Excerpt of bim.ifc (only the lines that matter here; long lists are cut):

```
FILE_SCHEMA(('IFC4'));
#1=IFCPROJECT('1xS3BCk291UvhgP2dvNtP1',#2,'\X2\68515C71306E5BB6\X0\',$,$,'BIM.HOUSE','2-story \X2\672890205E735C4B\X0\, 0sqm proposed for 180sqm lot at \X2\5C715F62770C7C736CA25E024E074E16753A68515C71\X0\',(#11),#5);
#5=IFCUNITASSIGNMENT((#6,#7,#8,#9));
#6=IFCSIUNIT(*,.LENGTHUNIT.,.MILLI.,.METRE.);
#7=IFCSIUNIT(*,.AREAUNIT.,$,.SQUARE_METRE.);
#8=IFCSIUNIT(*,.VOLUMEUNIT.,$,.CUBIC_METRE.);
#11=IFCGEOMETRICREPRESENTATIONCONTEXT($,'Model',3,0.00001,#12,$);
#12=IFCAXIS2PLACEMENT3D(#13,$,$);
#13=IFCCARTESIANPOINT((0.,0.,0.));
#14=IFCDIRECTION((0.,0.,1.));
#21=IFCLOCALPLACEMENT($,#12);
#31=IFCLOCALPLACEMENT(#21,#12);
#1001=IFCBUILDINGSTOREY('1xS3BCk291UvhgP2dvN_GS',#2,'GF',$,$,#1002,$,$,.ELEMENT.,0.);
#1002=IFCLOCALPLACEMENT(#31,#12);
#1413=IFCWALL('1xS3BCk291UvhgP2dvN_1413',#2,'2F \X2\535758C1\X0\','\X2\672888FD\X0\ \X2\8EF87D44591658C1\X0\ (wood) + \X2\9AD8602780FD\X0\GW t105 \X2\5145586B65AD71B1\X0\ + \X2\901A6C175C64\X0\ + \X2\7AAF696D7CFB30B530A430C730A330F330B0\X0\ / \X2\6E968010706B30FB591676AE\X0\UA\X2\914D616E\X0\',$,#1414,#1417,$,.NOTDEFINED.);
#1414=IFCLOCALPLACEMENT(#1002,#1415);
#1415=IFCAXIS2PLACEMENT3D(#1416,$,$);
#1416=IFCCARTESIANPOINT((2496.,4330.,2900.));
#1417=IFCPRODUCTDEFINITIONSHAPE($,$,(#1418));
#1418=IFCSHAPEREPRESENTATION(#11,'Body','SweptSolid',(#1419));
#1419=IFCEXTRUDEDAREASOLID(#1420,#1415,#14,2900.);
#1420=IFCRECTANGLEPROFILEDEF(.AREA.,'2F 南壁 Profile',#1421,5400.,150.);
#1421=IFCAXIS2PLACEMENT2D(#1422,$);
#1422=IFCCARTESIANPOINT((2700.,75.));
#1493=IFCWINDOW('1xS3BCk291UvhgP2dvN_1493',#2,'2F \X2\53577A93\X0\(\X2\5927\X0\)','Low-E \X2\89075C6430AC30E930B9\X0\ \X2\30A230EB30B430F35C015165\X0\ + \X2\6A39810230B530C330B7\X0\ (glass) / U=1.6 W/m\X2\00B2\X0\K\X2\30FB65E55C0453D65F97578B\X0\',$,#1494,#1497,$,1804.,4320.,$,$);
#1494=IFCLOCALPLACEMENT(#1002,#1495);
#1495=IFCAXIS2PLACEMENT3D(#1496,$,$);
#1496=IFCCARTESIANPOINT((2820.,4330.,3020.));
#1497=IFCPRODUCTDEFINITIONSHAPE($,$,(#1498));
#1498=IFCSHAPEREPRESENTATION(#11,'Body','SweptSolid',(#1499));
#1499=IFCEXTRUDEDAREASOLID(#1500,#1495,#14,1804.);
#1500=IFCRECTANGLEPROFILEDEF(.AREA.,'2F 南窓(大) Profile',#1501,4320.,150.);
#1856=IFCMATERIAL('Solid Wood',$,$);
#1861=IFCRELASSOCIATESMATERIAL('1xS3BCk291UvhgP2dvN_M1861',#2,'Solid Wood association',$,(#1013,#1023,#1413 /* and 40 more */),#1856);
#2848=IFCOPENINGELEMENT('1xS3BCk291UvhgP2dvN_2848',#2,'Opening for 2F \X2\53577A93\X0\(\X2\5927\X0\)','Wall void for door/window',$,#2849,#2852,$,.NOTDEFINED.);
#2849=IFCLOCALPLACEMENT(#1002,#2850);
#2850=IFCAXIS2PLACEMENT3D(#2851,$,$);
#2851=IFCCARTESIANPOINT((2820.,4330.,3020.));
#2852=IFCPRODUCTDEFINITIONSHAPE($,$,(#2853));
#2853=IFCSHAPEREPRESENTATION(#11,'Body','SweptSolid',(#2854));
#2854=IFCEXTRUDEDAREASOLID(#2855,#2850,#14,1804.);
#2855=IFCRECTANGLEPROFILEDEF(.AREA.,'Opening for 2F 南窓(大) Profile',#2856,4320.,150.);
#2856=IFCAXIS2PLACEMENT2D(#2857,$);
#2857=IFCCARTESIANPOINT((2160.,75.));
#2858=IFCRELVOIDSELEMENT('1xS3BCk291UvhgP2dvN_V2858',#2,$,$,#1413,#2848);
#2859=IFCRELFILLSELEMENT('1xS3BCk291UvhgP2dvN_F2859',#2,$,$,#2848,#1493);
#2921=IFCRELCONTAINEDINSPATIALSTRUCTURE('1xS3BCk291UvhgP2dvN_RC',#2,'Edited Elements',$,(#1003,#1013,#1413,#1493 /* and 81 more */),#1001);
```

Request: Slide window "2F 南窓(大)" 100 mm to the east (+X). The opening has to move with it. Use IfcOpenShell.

```python
import ifcopenshell
import ifcopenshell.api.geometry
import ifcopenshell.util.placement

model = ifcopenshell.open("bim.ifc")

window = model.by_guid("1xS3BCk291UvhgP2dvN_1493")
opening = window.FillsVoids[0].RelatingOpeningElement
wall = opening.VoidsElements[0].RelatingBuildingElement

wall_matrix = ifcopenshell.util.placement.get_local_placement(wall.ObjectPlacement)
shift = wall_matrix[:3, 0] * 100.0
before = ifcopenshell.util.placement.get_local_placement(window.ObjectPlacement)[:3, 3].copy()

# The window is not placed relative to its opening, so move both.
for product in (opening, window):
    matrix = ifcopenshell.util.placement.get_local_placement(product.ObjectPlacement)
    matrix[:3, 3] += shift
    ifcopenshell.api.geometry.edit_object_placement(model, product=product, matrix=matrix, is_si=False)

after = ifcopenshell.util.placement.get_local_placement(window.ObjectPlacement)[:3, 3]
print("window moved by", (after - before).round(3) + 0.0)

model.write("bim_rev.ifc")
```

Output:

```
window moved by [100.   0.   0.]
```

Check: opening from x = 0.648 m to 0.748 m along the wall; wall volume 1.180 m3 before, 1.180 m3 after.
